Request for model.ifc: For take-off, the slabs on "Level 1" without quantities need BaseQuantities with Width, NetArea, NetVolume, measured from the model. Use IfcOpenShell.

First a look at what the model holds.

```python
import ifcopenshell
import ifcopenshell.util.element
import ifcopenshell.util.unit

model = ifcopenshell.open("model.ifc")
print(model.schema)
for unit_type in ("LENGTHUNIT", "AREAUNIT", "VOLUMEUNIT"):
    print(unit_type, ifcopenshell.util.unit.calculate_unit_scale(model, unit_type))
storey = next(s for s in model.by_type("IfcBuildingStorey") if s.Name == "Level 1")
slabs = [e for e in ifcopenshell.util.element.get_decomposition(storey) if e.is_a("IfcSlab")]
for e in sorted(slabs, key=lambda e: e.id()):
    print(e.id(), e.is_a(), e.Name, list(ifcopenshell.util.element.get_psets(e, qtos_only=True)), sep=" | ")
```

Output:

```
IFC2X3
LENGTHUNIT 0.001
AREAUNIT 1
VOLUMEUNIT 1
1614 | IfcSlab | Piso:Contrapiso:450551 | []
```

```python
import ifcopenshell
import ifcopenshell.api.pset
import ifcopenshell.geom
import ifcopenshell.util.element
import ifcopenshell.util.shape
import ifcopenshell.util.unit

model = ifcopenshell.open("model.ifc")
unit_scale = ifcopenshell.util.unit.calculate_unit_scale(model)
area_scale = ifcopenshell.util.unit.calculate_unit_scale(model, "AREAUNIT")
volume_scale = ifcopenshell.util.unit.calculate_unit_scale(model, "VOLUMEUNIT")
settings = ifcopenshell.geom.settings()

storey = next(s for s in model.by_type("IfcBuildingStorey") if s.Name == "Level 1")
slabs = [e for e in ifcopenshell.util.element.get_decomposition(storey) if e.is_a("IfcSlab")]

for e in sorted(slabs, key=lambda e: e.id()):
    if ifcopenshell.util.element.get_psets(e, qtos_only=True, should_inherit=False):
        continue
    # Geometry comes back in metres, in the element's own axes.
    shape = ifcopenshell.geom.create_shape(settings, e)
    values = {
        "Width": ifcopenshell.util.shape.get_z(shape.geometry) / unit_scale,
        "NetArea": ifcopenshell.util.shape.get_footprint_area(shape.geometry) / area_scale,
        "NetVolume": ifcopenshell.util.shape.get_volume(shape.geometry) / volume_scale,
    }
    qto = ifcopenshell.api.pset.add_qto(model, product=e, name="BaseQuantities")
    ifcopenshell.api.pset.edit_qto(model, qto=qto, properties=values)
    print(e.id(), {k: round(v, 3) for k, v in values.items()})

model.write("model_rev.ifc")
```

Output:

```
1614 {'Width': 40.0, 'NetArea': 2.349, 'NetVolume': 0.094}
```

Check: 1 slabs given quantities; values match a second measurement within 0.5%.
